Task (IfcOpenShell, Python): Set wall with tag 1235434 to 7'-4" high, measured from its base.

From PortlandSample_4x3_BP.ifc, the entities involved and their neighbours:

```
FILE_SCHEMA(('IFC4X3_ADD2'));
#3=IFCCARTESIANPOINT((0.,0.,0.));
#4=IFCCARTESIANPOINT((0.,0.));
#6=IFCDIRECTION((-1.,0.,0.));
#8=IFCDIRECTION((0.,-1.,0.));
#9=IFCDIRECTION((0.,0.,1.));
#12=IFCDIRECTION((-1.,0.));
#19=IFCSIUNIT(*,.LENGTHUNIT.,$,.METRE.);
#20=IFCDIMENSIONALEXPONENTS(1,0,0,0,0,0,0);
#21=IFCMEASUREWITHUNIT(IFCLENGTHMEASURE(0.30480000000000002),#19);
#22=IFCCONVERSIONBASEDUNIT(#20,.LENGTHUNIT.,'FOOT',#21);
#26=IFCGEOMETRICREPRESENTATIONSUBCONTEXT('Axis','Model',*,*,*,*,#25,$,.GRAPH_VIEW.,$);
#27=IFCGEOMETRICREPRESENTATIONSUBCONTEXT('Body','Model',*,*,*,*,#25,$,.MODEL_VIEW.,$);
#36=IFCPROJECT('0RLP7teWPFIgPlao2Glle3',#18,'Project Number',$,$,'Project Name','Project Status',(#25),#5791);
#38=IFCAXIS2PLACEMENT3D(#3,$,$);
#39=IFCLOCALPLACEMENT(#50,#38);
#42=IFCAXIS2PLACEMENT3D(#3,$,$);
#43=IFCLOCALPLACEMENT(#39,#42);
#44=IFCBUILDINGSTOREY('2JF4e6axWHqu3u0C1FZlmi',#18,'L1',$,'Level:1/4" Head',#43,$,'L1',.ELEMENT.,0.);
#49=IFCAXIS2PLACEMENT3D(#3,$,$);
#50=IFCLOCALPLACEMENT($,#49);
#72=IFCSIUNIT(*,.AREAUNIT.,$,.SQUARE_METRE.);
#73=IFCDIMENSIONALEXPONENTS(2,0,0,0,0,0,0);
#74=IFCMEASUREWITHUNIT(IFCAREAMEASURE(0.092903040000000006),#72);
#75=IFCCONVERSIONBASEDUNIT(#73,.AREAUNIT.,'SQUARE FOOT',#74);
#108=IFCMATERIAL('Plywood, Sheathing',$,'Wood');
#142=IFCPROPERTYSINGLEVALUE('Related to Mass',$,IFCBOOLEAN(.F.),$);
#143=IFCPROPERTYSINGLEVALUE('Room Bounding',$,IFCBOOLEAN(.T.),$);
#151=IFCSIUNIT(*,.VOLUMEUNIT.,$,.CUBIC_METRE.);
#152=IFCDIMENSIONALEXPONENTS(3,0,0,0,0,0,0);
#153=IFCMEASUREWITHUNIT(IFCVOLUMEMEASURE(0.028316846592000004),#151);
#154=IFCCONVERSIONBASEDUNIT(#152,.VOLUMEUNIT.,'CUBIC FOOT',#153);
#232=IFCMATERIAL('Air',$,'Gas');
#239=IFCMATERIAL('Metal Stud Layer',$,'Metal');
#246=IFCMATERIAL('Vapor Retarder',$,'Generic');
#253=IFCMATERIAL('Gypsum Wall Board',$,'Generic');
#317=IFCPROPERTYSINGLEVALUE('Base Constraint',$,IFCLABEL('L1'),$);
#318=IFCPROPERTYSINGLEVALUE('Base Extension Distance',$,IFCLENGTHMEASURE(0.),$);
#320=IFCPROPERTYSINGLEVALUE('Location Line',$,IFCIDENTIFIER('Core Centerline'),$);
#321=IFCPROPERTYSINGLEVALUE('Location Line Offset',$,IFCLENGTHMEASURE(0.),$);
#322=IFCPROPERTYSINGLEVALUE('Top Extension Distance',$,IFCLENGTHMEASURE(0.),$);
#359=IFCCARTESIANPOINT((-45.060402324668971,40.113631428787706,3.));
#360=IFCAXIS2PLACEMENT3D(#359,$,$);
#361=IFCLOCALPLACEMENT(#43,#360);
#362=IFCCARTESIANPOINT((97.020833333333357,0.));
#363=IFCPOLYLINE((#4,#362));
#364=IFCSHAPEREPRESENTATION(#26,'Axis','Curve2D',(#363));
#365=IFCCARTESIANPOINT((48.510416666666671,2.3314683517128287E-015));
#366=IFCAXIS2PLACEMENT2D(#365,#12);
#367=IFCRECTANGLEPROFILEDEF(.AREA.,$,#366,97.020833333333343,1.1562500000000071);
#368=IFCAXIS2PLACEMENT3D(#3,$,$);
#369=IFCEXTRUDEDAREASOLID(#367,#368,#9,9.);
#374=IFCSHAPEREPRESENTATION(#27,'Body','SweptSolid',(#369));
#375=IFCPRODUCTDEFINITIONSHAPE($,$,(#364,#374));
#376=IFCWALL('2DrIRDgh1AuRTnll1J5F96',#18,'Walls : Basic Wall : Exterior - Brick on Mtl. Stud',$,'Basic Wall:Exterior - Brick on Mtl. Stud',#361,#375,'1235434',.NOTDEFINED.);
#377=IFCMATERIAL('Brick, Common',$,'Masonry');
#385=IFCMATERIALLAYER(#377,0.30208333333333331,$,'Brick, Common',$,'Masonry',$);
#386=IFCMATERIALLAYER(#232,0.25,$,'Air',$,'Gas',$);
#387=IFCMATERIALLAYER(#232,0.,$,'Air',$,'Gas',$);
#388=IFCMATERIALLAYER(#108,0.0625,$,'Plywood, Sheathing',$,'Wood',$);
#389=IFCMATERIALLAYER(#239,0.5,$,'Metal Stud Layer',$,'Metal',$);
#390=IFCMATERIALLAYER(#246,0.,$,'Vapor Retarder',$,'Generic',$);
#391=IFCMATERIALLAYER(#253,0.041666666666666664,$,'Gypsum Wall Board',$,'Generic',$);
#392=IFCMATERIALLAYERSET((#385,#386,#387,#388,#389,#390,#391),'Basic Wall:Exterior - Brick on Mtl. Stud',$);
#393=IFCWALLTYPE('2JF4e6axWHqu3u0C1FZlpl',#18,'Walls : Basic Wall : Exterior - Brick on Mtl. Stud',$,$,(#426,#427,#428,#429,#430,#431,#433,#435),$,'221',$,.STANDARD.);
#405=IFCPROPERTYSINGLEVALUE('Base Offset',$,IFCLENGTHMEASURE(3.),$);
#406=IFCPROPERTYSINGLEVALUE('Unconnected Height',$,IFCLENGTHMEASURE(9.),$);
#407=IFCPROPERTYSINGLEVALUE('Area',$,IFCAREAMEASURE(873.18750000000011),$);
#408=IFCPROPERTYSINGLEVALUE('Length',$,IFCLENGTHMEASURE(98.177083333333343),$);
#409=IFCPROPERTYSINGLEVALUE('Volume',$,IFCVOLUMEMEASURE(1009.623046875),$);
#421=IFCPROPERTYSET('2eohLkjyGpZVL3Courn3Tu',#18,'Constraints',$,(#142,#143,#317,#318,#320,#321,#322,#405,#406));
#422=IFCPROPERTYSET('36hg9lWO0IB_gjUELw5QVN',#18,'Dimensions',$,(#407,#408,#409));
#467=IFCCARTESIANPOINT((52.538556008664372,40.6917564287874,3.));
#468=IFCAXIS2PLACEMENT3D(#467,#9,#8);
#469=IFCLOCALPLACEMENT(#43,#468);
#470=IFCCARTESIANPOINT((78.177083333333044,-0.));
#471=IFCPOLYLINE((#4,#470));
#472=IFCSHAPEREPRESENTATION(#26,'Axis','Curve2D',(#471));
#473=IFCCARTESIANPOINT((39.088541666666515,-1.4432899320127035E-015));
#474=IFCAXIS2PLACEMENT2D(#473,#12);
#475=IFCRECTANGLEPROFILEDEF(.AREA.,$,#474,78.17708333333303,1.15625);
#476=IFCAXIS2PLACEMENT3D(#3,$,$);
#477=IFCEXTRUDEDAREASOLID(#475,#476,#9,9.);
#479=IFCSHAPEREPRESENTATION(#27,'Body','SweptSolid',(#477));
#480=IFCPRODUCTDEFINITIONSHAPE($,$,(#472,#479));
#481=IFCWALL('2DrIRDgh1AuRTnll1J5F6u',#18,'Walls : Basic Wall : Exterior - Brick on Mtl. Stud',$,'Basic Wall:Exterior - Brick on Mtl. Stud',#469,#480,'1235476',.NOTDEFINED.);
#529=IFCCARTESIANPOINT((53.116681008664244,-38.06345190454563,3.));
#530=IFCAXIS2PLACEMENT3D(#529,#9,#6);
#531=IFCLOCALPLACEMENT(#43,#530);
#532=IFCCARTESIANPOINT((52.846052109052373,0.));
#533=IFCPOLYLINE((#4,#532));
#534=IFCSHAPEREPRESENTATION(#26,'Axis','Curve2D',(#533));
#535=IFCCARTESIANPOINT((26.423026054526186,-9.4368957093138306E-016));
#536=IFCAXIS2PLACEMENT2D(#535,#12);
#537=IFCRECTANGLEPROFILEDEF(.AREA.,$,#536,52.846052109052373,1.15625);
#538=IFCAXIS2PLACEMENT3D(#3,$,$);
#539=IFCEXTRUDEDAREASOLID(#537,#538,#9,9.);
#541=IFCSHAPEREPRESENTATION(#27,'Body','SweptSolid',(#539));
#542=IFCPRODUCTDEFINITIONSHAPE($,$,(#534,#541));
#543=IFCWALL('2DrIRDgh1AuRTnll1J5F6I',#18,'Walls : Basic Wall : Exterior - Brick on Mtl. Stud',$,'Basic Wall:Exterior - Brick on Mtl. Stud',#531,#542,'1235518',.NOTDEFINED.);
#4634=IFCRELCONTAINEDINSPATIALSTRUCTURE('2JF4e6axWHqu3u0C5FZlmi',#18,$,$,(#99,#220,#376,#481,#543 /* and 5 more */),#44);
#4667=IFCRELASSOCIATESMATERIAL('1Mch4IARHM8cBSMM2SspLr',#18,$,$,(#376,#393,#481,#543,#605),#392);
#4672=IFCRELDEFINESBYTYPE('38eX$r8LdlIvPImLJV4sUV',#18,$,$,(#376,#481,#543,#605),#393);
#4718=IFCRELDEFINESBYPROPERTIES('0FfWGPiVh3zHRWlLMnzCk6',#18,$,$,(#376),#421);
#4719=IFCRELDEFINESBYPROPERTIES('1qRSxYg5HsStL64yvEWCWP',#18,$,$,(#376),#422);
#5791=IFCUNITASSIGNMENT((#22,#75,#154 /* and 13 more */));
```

```python
import ifcopenshell
import ifcopenshell.api.pset
import ifcopenshell.geom
import ifcopenshell.util.element
import ifcopenshell.util.representation
import ifcopenshell.util.shape
import ifcopenshell.util.unit

model = ifcopenshell.open("PortlandSample_4x3_BP.ifc")
unit_scale = ifcopenshell.util.unit.calculate_unit_scale(model)
area_scale = ifcopenshell.util.unit.calculate_unit_scale(model, "AREAUNIT")
volume_scale = ifcopenshell.util.unit.calculate_unit_scale(model, "VOLUMEUNIT")
settings = ifcopenshell.geom.settings()


def volume(element):
    """Net volume in cubic metres, openings subtracted."""
    shape = ifcopenshell.geom.create_shape(settings, element)
    return ifcopenshell.util.shape.get_volume(shape.geometry)


wall = model.by_guid("2DrIRDgh1AuRTnll1J5F96")
before = volume(wall)

body = ifcopenshell.util.representation.get_representation(wall, "Model", "Body")
solid = body.Items[0]
old_height = solid.Depth
solid.Depth = 88 * 0.0254 / unit_scale
after = volume(wall)
thickness = 0.3524  # wall thickness in metres

# Update the stored height, areas and volumes.
pset = model.by_id(ifcopenshell.util.element.get_pset(wall, "Constraints", should_inherit=False)["id"])
ifcopenshell.api.pset.edit_pset(model, pset=pset, properties={
    "Unconnected Height": model.create_entity("IfcLengthMeasure", solid.Depth),
})
pset = model.by_id(ifcopenshell.util.element.get_pset(wall, "Dimensions", should_inherit=False)["id"])
ifcopenshell.api.pset.edit_pset(model, pset=pset, properties={
    "Area": model.create_entity("IfcAreaMeasure", after / thickness / area_scale),
    "Volume": model.create_entity("IfcVolumeMeasure", after / volume_scale),
})

print(f"height {old_height:g} -> {solid.Depth:g}, volume {before:.3f} -> {after:.3f} m3")

model.write("PortlandSample_4x3_BP_updated.ifc")
```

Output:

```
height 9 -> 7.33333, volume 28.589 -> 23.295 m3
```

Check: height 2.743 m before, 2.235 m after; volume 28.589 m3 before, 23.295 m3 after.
